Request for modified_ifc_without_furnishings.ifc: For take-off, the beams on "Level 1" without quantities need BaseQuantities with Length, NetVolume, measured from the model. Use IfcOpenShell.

First a look at what the model holds.

```python
import ifcopenshell
import ifcopenshell.util.element
import ifcopenshell.util.unit

model = ifcopenshell.open("modified_ifc_without_furnishings.ifc")
print(model.schema)
for unit_type in ("LENGTHUNIT", "AREAUNIT", "VOLUMEUNIT"):
    print(unit_type, ifcopenshell.util.unit.calculate_unit_scale(model, unit_type))
storey = next(s for s in model.by_type("IfcBuildingStorey") if s.Name == "Level 1")
beams = [e for e in ifcopenshell.util.element.get_decomposition(storey) if e.is_a("IfcBeam")]
for e in sorted(beams, key=lambda e: e.id()):
    print(e.id(), e.is_a(), e.Name, list(ifcopenshell.util.element.get_psets(e, qtos_only=True)), sep=" | ")
```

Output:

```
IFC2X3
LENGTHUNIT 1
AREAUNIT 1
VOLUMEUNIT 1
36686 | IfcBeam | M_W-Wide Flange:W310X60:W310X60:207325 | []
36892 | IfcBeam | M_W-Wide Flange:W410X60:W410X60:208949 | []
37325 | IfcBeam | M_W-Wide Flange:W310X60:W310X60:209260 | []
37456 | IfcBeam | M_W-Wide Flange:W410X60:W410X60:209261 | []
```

```python
import ifcopenshell
import ifcopenshell.api.pset
import ifcopenshell.geom
import ifcopenshell.util.element
import ifcopenshell.util.shape
import ifcopenshell.util.unit

model = ifcopenshell.open("modified_ifc_without_furnishings.ifc")
unit_scale = ifcopenshell.util.unit.calculate_unit_scale(model)
volume_scale = ifcopenshell.util.unit.calculate_unit_scale(model, "VOLUMEUNIT")
settings = ifcopenshell.geom.settings()

storey = next(s for s in model.by_type("IfcBuildingStorey") if s.Name == "Level 1")
beams = [e for e in ifcopenshell.util.element.get_decomposition(storey) if e.is_a("IfcBeam")]

for e in sorted(beams, key=lambda e: e.id()):
    if ifcopenshell.util.element.get_psets(e, qtos_only=True, should_inherit=False):
        continue
    # Geometry comes back in metres, in the element's own axes.
    shape = ifcopenshell.geom.create_shape(settings, e)
    values = {
        "Length": ifcopenshell.util.shape.get_max_xyz(shape.geometry) / unit_scale,
        "NetVolume": ifcopenshell.util.shape.get_volume(shape.geometry) / volume_scale,
    }
    qto = ifcopenshell.api.pset.add_qto(model, product=e, name="BaseQuantities")
    ifcopenshell.api.pset.edit_qto(model, qto=qto, properties=values)
    print(e.id(), {k: round(v, 3) for k, v in values.items()})

model.write("modified_ifc_without_furnishings_edited.ifc")
```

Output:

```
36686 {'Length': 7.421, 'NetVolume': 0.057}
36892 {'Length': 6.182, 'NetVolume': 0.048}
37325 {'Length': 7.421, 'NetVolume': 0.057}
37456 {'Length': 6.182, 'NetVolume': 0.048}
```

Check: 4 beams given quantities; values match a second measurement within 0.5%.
